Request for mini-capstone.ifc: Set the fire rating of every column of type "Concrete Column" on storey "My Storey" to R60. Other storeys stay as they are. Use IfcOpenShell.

First a look at what the model holds.

```python
import ifcopenshell
import ifcopenshell.util.element

model = ifcopenshell.open("mini-capstone.ifc")
print(model.schema)
storey = next(s for s in model.by_type("IfcBuildingStorey") if s.Name == "My Storey")
columns = [e for e in ifcopenshell.util.element.get_decomposition(storey) if e.is_a("IfcColumn")]
seen = {}
for e in columns:
    element_type = ifcopenshell.util.element.get_type(e)
    key = (element_type.Name if element_type != e and element_type else None, ifcopenshell.util.element.get_pset(e, "Pset_ColumnCommon", "FireRating"))
    seen[key] = seen.get(key, 0) + 1
for (name, value), count in sorted(seen.items(), key=str):
    print(count, "x", name, "|", value)
```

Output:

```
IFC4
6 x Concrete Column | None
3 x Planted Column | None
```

```python
import ifcopenshell
import ifcopenshell.api.pset
import ifcopenshell.util.element

model = ifcopenshell.open("mini-capstone.ifc")

storey = next(s for s in model.by_type("IfcBuildingStorey") if s.Name == "My Storey")
columns = [e for e in ifcopenshell.util.element.get_decomposition(storey) if e.is_a("IfcColumn")]

count = 0
for e in columns:
    element_type = ifcopenshell.util.element.get_type(e)
    if element_type in (None, e) or element_type.Name != "Concrete Column":
        continue
    # add_pset returns the element's existing set when there is one.
    pset = ifcopenshell.api.pset.add_pset(model, product=e, name="Pset_ColumnCommon")
    ifcopenshell.api.pset.edit_pset(model, pset=pset, properties={"FireRating": "R60"})
    count += 1

print(count, "columns updated")

model.write("mini-capstone-out.ifc")
```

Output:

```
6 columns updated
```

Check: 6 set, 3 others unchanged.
